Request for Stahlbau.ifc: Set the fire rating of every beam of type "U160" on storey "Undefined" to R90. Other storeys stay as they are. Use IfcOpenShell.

First a look at what the model holds.

```python
import ifcopenshell
import ifcopenshell.util.element

model = ifcopenshell.open("Stahlbau.ifc")
print(model.schema)
storey = next(s for s in model.by_type("IfcBuildingStorey") if s.Name == "Undefined")
beams = [e for e in ifcopenshell.util.element.get_decomposition(storey) if e.is_a("IfcBeam")]
seen = {}
for e in beams:
    element_type = ifcopenshell.util.element.get_type(e)
    key = (element_type.Name if element_type != e and element_type else None, ifcopenshell.util.element.get_pset(e, "Pset_BeamCommon", "FireRating"))
    seen[key] = seen.get(key, 0) + 1
for (name, value), count in sorted(seen.items(), key=str):
    print(count, "x", name, "|", value)
```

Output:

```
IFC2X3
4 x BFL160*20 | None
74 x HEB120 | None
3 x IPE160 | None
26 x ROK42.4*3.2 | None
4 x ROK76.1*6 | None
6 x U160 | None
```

```python
import ifcopenshell
import ifcopenshell.api.pset
import ifcopenshell.util.element

model = ifcopenshell.open("Stahlbau.ifc")

storey = next(s for s in model.by_type("IfcBuildingStorey") if s.Name == "Undefined")
beams = [e for e in ifcopenshell.util.element.get_decomposition(storey) if e.is_a("IfcBeam")]

count = 0
for e in beams:
    element_type = ifcopenshell.util.element.get_type(e)
    if element_type in (None, e) or element_type.Name != "U160":
        continue
    # add_pset returns the element's existing set when there is one.
    pset = ifcopenshell.api.pset.add_pset(model, product=e, name="Pset_BeamCommon")
    ifcopenshell.api.pset.edit_pset(model, pset=pset, properties={"FireRating": "R90"})
    count += 1

print(count, "beams updated")

model.write("Stahlbau_rev.ifc")
```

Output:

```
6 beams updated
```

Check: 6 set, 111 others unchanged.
